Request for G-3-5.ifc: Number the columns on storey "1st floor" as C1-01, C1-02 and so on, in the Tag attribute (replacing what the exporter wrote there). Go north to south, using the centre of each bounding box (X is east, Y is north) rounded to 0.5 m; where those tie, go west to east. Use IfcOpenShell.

First a look at what the model holds.

```python
import ifcopenshell
import ifcopenshell.util.element
import ifcopenshell.util.placement

model = ifcopenshell.open("G-3-5.ifc")
print(model.schema)
storey = next(s for s in model.by_type("IfcBuildingStorey") if s.Name == "1st floor")
columns = [e for e in ifcopenshell.util.element.get_decomposition(storey) if e.is_a("IfcColumn")]
for e in sorted(columns, key=lambda e: e.id()):
    origin = ifcopenshell.util.placement.get_local_placement(e.ObjectPlacement)[:3, 3]
    print(e.id(), e.Tag, e.Name, origin.round(2) + 0.0, sep=" | ")
```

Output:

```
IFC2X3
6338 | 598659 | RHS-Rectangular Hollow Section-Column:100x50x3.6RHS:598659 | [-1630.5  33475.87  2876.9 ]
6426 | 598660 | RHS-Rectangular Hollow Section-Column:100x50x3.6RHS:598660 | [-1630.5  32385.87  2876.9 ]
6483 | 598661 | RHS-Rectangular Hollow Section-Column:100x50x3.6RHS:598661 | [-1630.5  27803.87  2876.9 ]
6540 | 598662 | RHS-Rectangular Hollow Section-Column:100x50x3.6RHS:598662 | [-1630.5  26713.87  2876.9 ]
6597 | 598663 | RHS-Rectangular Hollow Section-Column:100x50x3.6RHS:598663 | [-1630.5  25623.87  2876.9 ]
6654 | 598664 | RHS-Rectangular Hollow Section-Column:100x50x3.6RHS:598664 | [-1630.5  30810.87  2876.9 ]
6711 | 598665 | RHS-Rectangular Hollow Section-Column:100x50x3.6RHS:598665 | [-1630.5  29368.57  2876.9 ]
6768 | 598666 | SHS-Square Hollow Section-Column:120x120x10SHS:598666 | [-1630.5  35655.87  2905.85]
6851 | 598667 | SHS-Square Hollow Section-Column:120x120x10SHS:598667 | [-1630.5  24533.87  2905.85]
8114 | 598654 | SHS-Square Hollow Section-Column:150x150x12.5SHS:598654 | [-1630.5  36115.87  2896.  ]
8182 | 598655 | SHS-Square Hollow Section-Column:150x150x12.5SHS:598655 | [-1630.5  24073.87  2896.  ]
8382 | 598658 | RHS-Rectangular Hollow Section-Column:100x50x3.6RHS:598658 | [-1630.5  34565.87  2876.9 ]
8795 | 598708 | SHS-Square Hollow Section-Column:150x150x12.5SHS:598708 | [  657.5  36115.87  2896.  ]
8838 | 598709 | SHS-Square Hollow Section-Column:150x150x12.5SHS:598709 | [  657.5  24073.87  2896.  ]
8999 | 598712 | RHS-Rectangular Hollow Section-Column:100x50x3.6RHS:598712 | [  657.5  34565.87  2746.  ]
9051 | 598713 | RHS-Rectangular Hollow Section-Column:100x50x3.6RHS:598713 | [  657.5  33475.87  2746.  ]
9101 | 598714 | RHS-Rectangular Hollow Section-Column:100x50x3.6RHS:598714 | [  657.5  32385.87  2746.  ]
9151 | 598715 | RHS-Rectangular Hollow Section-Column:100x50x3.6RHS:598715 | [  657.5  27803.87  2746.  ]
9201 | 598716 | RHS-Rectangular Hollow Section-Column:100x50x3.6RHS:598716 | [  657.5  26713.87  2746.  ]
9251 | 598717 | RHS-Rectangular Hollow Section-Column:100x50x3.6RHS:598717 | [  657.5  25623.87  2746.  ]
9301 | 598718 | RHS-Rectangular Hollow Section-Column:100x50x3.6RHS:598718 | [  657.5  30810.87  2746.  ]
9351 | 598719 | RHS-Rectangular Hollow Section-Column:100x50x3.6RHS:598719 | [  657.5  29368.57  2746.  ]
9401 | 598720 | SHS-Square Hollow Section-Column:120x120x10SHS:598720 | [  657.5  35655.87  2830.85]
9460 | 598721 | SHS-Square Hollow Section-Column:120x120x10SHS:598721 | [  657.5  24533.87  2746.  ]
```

```python
import ifcopenshell
import ifcopenshell.geom
import ifcopenshell.util.element
import ifcopenshell.util.shape

model = ifcopenshell.open("G-3-5.ifc")
settings = ifcopenshell.geom.settings()
settings.set("use-world-coords", True)


def centre(element):
    shape = ifcopenshell.geom.create_shape(settings, element)
    return ifcopenshell.util.shape.get_bbox_centroid(shape.geometry)


storey = next(s for s in model.by_type("IfcBuildingStorey") if s.Name == "1st floor")
columns = [e for e in ifcopenshell.util.element.get_decomposition(storey) if e.is_a("IfcColumn")]

# Insertion points can sit at a corner or the storey origin, so sort by the geometry (in metres).
centres = {e: centre(e) for e in columns}
columns.sort(key=lambda e: (-round(centres[e][1] / 0.5), centres[e][0]))

for i, e in enumerate(columns, start=1):
    number = f"C1-{i:02d}"
    e.Tag = number
    print(e.id(), number)

model.write("G-3-5_rev.ifc")
```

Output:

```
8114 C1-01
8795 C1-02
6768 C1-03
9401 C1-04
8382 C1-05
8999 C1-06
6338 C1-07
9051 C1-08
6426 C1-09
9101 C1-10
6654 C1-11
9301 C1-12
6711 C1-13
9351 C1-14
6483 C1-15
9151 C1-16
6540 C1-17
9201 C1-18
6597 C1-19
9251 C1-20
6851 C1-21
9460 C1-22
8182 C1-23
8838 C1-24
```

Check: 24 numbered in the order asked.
